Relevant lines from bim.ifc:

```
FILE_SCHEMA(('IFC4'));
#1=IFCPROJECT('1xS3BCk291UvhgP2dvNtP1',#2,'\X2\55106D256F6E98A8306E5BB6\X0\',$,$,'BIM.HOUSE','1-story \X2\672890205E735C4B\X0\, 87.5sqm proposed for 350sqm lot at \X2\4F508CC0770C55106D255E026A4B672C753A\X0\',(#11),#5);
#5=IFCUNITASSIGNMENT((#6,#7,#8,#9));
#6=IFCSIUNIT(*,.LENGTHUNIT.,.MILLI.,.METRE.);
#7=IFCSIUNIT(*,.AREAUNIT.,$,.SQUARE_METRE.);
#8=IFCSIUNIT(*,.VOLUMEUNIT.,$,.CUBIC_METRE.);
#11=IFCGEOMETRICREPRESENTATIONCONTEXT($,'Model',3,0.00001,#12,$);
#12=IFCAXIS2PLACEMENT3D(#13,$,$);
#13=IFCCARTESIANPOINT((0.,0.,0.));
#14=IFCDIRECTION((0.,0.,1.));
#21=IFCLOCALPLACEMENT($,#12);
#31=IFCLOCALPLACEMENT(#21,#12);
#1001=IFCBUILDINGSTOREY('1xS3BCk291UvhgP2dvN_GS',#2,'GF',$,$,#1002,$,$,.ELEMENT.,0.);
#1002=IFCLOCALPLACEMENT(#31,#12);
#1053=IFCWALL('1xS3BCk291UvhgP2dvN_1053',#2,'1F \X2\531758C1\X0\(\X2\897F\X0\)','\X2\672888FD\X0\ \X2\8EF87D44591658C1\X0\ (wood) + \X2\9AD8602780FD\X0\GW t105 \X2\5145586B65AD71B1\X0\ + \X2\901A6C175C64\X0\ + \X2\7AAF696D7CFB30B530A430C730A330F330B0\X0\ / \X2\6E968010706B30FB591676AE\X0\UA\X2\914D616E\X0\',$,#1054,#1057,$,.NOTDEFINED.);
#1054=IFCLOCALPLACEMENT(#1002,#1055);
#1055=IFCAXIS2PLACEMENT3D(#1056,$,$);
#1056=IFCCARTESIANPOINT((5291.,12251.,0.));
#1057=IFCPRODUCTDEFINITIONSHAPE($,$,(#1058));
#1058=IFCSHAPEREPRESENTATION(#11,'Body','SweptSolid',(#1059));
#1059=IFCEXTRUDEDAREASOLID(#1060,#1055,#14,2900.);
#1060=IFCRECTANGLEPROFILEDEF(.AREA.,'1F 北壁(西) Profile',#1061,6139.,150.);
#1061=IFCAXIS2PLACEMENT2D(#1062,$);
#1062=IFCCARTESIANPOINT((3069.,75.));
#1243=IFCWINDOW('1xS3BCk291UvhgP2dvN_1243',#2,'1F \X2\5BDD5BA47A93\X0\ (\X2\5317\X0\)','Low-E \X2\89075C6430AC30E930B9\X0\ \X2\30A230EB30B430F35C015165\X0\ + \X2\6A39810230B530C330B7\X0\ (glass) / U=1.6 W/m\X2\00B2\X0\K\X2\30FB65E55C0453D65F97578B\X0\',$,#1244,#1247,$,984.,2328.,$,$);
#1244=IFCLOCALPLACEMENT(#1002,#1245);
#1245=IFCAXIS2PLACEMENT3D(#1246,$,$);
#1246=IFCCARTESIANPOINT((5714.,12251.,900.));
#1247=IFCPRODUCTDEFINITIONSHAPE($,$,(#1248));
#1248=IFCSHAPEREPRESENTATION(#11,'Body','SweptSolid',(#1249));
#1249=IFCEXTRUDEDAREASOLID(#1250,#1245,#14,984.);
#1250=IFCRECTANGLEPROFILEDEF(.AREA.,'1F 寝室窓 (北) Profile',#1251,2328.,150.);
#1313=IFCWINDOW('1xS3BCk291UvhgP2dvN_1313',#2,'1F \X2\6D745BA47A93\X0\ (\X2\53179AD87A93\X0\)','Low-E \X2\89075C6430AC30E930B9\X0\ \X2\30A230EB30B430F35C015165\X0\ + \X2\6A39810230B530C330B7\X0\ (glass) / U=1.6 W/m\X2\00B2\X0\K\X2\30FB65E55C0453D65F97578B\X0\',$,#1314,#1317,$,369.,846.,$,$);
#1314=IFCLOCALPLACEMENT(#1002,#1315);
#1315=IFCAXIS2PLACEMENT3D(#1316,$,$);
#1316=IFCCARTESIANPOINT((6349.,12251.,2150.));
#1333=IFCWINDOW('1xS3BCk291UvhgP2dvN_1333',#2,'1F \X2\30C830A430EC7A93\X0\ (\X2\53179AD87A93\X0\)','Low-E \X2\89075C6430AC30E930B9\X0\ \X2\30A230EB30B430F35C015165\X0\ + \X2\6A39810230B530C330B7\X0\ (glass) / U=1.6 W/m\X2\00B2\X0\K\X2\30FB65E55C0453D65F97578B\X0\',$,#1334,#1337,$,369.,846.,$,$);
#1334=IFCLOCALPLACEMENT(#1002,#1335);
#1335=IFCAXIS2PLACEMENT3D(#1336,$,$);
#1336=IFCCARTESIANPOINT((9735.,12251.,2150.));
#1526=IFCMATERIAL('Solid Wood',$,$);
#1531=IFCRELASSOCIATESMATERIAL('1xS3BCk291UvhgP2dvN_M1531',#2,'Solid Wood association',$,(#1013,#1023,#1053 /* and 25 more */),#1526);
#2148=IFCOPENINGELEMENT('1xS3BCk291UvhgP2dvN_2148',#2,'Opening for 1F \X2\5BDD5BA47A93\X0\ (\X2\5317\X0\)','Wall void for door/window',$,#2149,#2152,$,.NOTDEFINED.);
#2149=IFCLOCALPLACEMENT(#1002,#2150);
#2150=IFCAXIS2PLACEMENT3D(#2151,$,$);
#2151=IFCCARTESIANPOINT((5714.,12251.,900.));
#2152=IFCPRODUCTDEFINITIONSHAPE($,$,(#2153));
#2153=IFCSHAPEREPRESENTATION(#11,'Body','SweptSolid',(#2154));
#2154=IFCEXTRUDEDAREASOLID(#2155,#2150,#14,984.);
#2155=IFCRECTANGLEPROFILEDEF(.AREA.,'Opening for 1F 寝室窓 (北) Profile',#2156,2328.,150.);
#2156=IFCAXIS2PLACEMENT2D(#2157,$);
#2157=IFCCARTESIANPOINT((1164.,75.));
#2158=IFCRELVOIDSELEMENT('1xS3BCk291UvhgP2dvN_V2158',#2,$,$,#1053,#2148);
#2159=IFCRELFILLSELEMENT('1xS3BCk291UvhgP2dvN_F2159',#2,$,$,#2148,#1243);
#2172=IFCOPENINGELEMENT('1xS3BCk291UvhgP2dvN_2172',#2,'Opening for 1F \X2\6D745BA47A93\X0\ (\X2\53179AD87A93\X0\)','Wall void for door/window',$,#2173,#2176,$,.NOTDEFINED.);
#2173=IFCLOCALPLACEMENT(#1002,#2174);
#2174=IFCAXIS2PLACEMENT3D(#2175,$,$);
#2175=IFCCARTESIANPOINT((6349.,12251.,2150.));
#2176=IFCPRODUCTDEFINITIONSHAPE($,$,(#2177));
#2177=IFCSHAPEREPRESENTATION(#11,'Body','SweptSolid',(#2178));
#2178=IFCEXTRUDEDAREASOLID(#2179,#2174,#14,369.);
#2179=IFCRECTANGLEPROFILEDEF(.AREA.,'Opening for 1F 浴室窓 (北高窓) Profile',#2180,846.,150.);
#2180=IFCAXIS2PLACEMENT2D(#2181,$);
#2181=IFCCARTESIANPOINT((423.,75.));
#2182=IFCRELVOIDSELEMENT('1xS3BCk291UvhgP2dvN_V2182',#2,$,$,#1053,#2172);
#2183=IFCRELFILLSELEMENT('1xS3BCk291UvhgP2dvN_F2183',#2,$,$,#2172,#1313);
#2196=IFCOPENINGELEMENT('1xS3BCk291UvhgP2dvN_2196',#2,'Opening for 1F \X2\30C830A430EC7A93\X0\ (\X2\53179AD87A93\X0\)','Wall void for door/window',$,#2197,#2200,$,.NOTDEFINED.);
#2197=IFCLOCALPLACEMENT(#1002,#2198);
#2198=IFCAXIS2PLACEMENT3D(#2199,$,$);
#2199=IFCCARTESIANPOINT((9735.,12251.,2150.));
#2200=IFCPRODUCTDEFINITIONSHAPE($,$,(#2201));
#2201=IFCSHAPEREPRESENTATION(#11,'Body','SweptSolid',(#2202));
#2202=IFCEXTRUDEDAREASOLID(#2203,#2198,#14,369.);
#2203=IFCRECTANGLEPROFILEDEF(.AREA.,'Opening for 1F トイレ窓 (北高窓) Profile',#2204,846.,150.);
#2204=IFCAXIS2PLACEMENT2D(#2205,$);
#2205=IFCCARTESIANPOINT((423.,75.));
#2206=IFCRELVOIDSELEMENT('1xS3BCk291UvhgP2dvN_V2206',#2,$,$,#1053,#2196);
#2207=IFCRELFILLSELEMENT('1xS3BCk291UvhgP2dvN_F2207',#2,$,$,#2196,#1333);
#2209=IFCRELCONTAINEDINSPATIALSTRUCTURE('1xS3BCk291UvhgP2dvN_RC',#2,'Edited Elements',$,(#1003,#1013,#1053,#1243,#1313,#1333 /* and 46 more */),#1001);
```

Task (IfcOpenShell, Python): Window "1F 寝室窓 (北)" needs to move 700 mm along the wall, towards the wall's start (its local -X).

```python
import ifcopenshell
import ifcopenshell.api.geometry
import ifcopenshell.util.placement
import ifcopenshell.util.unit

model = ifcopenshell.open("bim.ifc")
unit_scale = ifcopenshell.util.unit.calculate_unit_scale(model)

window = model.by_guid("1xS3BCk291UvhgP2dvN_1243")
opening = window.FillsVoids[0].RelatingOpeningElement
wall = opening.VoidsElements[0].RelatingBuildingElement

wall_matrix = ifcopenshell.util.placement.get_local_placement(wall.ObjectPlacement)
shift = wall_matrix[:3, 0] * -0.7 / unit_scale
before = ifcopenshell.util.placement.get_local_placement(window.ObjectPlacement)[:3, 3].copy()

# The window is not placed relative to its opening, so move both.
for product in (opening, window):
    matrix = ifcopenshell.util.placement.get_local_placement(product.ObjectPlacement)
    matrix[:3, 3] += shift
    ifcopenshell.api.geometry.edit_object_placement(model, product=product, matrix=matrix, is_si=False)

after = ifcopenshell.util.placement.get_local_placement(window.ObjectPlacement)[:3, 3]
print("window moved by", (after - before).round(3) + 0.0)

model.write("bim_edited.ifc")
```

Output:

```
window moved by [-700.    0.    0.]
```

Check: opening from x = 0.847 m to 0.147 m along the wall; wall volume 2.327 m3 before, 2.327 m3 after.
